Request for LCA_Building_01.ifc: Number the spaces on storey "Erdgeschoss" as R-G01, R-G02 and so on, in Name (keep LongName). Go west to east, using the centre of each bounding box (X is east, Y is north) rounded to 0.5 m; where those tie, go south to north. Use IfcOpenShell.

First a look at what the model holds.

```python
import ifcopenshell
import ifcopenshell.util.element
import ifcopenshell.util.placement

model = ifcopenshell.open("LCA_Building_01.ifc")
print(model.schema)
storey = next(s for s in model.by_type("IfcBuildingStorey") if s.Name == "Erdgeschoss")
spaces = [e for e in ifcopenshell.util.element.get_decomposition(storey) if e.is_a("IfcSpace")]
for e in sorted(spaces, key=lambda e: e.id()):
    origin = ifcopenshell.util.placement.get_local_placement(e.ObjectPlacement)[:3, 3]
    print(e.id(), e.Name, e.LongName, origin.round(2) + 0.0, sep=" | ")
```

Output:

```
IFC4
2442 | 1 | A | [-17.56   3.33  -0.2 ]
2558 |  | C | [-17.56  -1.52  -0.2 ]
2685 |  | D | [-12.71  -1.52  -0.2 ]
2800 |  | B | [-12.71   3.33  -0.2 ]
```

```python
import ifcopenshell
import ifcopenshell.geom
import ifcopenshell.util.element
import ifcopenshell.util.shape

model = ifcopenshell.open("LCA_Building_01.ifc")
settings = ifcopenshell.geom.settings()
settings.set("use-world-coords", True)


def centre(element):
    shape = ifcopenshell.geom.create_shape(settings, element)
    return ifcopenshell.util.shape.get_bbox_centroid(shape.geometry)


storey = next(s for s in model.by_type("IfcBuildingStorey") if s.Name == "Erdgeschoss")
spaces = [e for e in ifcopenshell.util.element.get_decomposition(storey) if e.is_a("IfcSpace")]

# Insertion points can sit at a corner or the storey origin, so sort by the geometry (in metres).
centres = {e: centre(e) for e in spaces}
spaces.sort(key=lambda e: (round(centres[e][0] / 0.5), centres[e][1]))

for i, e in enumerate(spaces, start=1):
    number = f"R-G{i:02d}"
    e.Name = number
    print(e.id(), number)

model.write("LCA_Building_01-out.ifc")
```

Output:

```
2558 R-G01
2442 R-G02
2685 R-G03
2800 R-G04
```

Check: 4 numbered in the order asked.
